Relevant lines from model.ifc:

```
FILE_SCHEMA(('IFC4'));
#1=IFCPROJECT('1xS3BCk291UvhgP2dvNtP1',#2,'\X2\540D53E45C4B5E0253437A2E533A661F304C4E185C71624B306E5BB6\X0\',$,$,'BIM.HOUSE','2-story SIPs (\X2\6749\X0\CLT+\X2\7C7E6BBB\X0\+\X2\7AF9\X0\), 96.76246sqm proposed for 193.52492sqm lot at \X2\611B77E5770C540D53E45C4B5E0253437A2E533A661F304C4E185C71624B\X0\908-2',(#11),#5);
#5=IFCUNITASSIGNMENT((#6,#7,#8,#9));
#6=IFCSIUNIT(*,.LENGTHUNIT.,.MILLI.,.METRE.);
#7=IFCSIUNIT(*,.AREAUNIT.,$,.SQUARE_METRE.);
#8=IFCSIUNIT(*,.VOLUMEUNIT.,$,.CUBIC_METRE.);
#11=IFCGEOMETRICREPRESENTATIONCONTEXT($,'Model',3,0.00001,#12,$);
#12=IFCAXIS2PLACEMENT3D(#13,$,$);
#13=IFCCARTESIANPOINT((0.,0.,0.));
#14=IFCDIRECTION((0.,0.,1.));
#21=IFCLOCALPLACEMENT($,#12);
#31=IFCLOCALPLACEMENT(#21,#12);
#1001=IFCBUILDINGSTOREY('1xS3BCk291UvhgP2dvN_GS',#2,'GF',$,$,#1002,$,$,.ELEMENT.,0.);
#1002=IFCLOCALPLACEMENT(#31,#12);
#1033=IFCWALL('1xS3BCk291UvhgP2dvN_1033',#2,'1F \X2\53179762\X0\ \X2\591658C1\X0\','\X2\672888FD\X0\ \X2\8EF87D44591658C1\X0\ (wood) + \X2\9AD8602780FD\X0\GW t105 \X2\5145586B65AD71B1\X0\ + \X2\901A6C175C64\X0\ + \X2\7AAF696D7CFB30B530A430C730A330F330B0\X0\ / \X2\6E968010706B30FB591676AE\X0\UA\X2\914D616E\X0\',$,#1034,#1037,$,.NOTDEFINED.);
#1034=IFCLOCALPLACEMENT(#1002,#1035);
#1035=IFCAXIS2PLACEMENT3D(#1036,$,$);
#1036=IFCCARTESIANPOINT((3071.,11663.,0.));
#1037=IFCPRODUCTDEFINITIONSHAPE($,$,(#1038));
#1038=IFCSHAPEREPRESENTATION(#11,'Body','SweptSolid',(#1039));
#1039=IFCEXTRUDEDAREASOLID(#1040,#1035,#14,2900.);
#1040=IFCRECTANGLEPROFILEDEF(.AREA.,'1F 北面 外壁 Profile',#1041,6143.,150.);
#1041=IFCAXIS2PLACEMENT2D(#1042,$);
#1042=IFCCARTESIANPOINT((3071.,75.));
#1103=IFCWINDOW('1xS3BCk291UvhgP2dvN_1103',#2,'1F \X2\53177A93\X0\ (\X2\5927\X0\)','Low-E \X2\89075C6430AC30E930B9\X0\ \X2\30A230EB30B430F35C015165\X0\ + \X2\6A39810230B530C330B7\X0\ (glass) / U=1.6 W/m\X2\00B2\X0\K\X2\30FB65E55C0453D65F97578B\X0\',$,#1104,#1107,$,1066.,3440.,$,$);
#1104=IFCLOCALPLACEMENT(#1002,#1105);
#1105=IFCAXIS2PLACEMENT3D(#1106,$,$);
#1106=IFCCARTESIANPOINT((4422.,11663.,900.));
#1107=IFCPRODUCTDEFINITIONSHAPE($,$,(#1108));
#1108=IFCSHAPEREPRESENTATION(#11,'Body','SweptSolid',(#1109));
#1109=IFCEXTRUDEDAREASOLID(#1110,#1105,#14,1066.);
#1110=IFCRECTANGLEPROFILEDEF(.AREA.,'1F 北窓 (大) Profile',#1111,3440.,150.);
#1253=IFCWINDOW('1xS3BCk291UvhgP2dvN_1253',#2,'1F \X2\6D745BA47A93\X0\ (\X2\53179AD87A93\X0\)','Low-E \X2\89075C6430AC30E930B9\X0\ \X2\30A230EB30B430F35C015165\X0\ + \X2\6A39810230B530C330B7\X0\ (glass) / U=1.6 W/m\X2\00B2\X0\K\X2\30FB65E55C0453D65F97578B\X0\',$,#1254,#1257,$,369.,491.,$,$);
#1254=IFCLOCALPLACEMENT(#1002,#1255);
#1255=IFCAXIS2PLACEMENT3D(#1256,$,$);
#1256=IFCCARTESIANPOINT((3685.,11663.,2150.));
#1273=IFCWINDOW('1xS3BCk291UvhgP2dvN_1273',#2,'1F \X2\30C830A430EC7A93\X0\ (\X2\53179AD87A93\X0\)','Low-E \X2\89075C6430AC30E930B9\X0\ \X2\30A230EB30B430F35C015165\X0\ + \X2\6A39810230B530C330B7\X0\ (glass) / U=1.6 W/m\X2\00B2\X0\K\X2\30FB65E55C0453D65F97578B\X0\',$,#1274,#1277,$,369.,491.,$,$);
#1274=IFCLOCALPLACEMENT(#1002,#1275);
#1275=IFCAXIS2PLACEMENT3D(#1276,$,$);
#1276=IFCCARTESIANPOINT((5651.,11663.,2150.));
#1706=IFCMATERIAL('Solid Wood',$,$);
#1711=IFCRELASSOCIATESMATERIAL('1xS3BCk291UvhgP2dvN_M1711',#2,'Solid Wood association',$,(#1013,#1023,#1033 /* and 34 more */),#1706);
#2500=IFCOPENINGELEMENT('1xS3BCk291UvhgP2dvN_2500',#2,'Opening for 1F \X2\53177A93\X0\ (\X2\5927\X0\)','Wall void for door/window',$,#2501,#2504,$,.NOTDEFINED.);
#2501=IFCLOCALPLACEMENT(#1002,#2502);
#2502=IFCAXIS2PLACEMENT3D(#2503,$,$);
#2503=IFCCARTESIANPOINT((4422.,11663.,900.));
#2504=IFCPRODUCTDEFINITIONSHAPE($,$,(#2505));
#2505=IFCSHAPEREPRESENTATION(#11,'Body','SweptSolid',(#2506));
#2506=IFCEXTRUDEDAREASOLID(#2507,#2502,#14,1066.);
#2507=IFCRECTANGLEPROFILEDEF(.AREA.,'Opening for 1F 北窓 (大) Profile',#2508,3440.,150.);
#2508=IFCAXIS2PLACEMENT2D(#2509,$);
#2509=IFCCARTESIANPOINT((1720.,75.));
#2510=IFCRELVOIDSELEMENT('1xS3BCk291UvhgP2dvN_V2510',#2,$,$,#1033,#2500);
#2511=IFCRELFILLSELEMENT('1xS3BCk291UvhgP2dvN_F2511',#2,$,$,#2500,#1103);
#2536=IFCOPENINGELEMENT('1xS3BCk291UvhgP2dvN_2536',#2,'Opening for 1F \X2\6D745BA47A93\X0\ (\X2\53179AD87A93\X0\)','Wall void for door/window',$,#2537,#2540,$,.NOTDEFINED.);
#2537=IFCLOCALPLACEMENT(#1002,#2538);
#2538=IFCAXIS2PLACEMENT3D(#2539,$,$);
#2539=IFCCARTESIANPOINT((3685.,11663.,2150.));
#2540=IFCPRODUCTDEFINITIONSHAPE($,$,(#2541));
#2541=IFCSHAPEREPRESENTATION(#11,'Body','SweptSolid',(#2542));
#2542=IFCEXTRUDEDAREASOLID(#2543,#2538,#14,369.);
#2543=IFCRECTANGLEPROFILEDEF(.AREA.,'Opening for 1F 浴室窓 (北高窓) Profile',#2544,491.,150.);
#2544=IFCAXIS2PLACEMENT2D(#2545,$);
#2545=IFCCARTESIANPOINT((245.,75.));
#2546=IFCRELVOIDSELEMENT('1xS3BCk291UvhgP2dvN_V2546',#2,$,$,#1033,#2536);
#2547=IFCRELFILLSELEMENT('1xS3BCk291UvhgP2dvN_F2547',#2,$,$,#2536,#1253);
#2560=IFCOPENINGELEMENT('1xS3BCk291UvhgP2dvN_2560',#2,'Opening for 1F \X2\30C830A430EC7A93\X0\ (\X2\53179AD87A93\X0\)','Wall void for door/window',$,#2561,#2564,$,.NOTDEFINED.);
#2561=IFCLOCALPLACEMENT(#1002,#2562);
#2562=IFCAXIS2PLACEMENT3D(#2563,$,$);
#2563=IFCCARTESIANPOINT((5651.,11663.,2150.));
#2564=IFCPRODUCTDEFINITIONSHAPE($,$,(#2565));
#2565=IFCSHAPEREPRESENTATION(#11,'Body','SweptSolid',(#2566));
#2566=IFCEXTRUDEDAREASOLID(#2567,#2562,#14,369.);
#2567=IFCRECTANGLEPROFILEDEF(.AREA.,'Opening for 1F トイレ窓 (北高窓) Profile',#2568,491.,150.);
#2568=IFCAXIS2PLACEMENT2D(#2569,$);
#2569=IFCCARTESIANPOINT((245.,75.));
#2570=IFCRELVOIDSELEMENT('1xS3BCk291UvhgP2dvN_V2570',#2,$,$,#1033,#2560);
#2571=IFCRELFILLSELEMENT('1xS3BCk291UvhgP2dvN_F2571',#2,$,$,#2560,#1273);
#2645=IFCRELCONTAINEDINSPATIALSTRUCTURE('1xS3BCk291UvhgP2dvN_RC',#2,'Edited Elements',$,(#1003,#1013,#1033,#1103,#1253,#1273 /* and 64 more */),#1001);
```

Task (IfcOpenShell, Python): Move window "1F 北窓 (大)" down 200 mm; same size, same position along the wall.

```python
import numpy as np
import ifcopenshell
import ifcopenshell.api.geometry
import ifcopenshell.util.placement
import ifcopenshell.util.unit

model = ifcopenshell.open("model.ifc")
unit_scale = ifcopenshell.util.unit.calculate_unit_scale(model)

window = model.by_guid("1xS3BCk291UvhgP2dvN_1103")
opening = window.FillsVoids[0].RelatingOpeningElement
dz = -0.2 / unit_scale

shift = np.array([0.0, 0.0, dz])
# The window is not placed relative to its opening, so move both.
for product in (opening, window):
    matrix = ifcopenshell.util.placement.get_local_placement(product.ObjectPlacement)
    matrix[:3, 3] += shift
    ifcopenshell.api.geometry.edit_object_placement(model, product=product, matrix=matrix, is_si=False)

print(f"moved by {dz * unit_scale:+.3f} m")

model.write("model_updated.ifc")
```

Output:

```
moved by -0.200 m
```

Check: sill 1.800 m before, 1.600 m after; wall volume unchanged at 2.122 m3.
